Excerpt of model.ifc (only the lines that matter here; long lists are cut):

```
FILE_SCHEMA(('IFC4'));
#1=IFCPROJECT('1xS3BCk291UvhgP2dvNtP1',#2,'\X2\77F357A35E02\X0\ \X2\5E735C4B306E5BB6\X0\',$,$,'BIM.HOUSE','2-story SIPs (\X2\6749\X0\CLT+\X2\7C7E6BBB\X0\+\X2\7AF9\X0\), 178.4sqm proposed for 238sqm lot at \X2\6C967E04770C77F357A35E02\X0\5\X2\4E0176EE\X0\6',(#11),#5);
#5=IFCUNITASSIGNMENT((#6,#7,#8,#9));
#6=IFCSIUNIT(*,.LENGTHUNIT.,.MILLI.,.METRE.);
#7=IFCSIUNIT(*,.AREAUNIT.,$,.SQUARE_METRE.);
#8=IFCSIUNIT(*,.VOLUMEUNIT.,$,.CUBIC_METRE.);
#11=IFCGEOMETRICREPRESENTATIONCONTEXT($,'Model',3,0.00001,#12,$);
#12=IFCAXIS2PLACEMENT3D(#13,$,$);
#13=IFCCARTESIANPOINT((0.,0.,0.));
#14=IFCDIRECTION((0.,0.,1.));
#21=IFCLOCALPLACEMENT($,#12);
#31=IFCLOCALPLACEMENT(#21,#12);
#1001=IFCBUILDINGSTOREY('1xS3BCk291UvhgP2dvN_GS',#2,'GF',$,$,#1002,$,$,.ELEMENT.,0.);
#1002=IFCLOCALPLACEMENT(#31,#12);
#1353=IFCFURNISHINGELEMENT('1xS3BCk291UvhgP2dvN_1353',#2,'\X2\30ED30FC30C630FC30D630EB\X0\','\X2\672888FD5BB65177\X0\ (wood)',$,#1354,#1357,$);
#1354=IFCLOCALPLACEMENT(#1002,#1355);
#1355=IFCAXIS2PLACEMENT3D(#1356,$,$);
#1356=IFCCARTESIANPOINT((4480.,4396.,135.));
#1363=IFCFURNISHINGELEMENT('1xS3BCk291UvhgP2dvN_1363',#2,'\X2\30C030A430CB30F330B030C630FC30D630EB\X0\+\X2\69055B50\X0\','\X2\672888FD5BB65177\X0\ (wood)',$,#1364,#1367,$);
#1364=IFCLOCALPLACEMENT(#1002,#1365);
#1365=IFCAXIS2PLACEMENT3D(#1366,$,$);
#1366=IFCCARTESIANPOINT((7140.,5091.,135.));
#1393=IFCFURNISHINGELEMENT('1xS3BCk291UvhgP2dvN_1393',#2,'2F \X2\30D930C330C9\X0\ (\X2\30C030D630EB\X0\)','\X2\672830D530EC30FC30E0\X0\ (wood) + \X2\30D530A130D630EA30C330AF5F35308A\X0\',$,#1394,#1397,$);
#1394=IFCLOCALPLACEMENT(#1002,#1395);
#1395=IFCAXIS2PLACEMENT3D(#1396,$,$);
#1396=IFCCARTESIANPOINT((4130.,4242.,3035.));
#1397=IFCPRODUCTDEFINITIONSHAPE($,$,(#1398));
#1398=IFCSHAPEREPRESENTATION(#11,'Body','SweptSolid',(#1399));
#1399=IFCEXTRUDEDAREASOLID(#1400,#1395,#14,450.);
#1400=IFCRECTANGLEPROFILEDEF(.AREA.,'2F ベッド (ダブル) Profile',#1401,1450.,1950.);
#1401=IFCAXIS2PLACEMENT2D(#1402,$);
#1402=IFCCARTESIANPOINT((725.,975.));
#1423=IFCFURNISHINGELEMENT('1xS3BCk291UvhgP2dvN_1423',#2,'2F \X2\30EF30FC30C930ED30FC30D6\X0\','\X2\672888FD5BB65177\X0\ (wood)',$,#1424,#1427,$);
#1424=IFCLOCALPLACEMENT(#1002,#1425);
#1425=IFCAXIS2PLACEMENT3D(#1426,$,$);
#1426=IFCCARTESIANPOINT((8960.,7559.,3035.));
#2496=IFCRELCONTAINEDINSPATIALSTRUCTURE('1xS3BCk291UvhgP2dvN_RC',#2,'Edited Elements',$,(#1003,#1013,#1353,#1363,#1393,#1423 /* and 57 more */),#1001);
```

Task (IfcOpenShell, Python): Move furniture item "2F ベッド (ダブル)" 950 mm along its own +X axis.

```python
import ifcopenshell
import ifcopenshell.api.geometry
import ifcopenshell.util.placement

model = ifcopenshell.open("model.ifc")

item = model.by_guid("1xS3BCk291UvhgP2dvN_1393")
matrix = ifcopenshell.util.placement.get_local_placement(item.ObjectPlacement)
matrix[:3, 3] += matrix[:3, 0] * 950.0
ifcopenshell.api.geometry.edit_object_placement(model, product=item, matrix=matrix, is_si=False)

print(ifcopenshell.util.placement.get_local_placement(item.ObjectPlacement).round(3) + 0.0)

model.write("model_edited.ifc")
```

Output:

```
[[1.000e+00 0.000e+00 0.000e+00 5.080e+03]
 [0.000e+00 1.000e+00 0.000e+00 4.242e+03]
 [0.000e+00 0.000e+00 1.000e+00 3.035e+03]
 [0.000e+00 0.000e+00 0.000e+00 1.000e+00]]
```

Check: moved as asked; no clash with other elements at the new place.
